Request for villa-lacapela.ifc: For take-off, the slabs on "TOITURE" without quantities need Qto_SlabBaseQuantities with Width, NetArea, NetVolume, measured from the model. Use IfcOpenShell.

First a look at what the model holds.

```python
import ifcopenshell
import ifcopenshell.util.element
import ifcopenshell.util.unit

model = ifcopenshell.open("villa-lacapela.ifc")
print(model.schema)
for unit_type in ("LENGTHUNIT", "AREAUNIT", "VOLUMEUNIT"):
    print(unit_type, ifcopenshell.util.unit.calculate_unit_scale(model, unit_type))
storey = next(s for s in model.by_type("IfcBuildingStorey") if s.Name == "TOITURE")
slabs = [e for e in ifcopenshell.util.element.get_decomposition(storey) if e.is_a("IfcSlab")]
for e in sorted(slabs, key=lambda e: e.id()):
    print(e.id(), e.is_a(), e.Name, list(ifcopenshell.util.element.get_psets(e, qtos_only=True)), sep=" | ")
```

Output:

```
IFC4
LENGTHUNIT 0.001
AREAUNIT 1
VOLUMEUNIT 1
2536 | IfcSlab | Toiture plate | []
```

```python
import ifcopenshell
import ifcopenshell.api.pset
import ifcopenshell.geom
import ifcopenshell.util.element
import ifcopenshell.util.shape
import ifcopenshell.util.unit

model = ifcopenshell.open("villa-lacapela.ifc")
unit_scale = ifcopenshell.util.unit.calculate_unit_scale(model)
area_scale = ifcopenshell.util.unit.calculate_unit_scale(model, "AREAUNIT")
volume_scale = ifcopenshell.util.unit.calculate_unit_scale(model, "VOLUMEUNIT")
settings = ifcopenshell.geom.settings()

storey = next(s for s in model.by_type("IfcBuildingStorey") if s.Name == "TOITURE")
slabs = [e for e in ifcopenshell.util.element.get_decomposition(storey) if e.is_a("IfcSlab")]

for e in sorted(slabs, key=lambda e: e.id()):
    if ifcopenshell.util.element.get_psets(e, qtos_only=True, should_inherit=False):
        continue
    # Geometry comes back in metres, in the element's own axes.
    shape = ifcopenshell.geom.create_shape(settings, e)
    values = {
        "Width": ifcopenshell.util.shape.get_z(shape.geometry) / unit_scale,
        "NetArea": ifcopenshell.util.shape.get_footprint_area(shape.geometry) / area_scale,
        "NetVolume": ifcopenshell.util.shape.get_volume(shape.geometry) / volume_scale,
    }
    qto = ifcopenshell.api.pset.add_qto(model, product=e, name="Qto_SlabBaseQuantities")
    ifcopenshell.api.pset.edit_qto(model, qto=qto, properties=values)
    print(e.id(), {k: round(v, 3) for k, v in values.items()})

model.write("villa-lacapela_updated.ifc")
```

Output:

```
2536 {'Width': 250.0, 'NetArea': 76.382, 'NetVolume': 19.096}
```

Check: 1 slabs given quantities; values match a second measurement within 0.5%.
